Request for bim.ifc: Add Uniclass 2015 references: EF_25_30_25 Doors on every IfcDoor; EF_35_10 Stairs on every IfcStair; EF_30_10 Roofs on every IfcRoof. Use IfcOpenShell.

First a look at what the model holds.

```python
import ifcopenshell

model = ifcopenshell.open("bim.ifc")
print(model.schema)
print("classifications:", [c.Name for c in model.by_type("IfcClassification")])
for ifc_class in ("IfcDoor", "IfcRoof", "IfcStair", "IfcWall", "IfcWindow"):
    print(ifc_class, len(model.by_type(ifc_class)))
```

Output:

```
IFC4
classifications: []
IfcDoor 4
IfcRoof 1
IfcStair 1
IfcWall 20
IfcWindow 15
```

```python
import ifcopenshell
import ifcopenshell.api.classification

model = ifcopenshell.open("bim.ifc")

system = ifcopenshell.api.classification.add_classification(model, classification="Uniclass 2015")

codes = {
    "IfcDoor": ("EF_25_30_25", "Doors"),
    "IfcStair": ("EF_35_10", "Stairs"),
    "IfcRoof": ("EF_30_10", "Roofs"),
}
for ifc_class, (code, name) in codes.items():
    products = model.by_type(ifc_class)
    ifcopenshell.api.classification.add_reference(
        model, products=products, classification=system, identification=code, name=name
    )
    print(code, len(products))

model.write("bim_v2.ifc")
```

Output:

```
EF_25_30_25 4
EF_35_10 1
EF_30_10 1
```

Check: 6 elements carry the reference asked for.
